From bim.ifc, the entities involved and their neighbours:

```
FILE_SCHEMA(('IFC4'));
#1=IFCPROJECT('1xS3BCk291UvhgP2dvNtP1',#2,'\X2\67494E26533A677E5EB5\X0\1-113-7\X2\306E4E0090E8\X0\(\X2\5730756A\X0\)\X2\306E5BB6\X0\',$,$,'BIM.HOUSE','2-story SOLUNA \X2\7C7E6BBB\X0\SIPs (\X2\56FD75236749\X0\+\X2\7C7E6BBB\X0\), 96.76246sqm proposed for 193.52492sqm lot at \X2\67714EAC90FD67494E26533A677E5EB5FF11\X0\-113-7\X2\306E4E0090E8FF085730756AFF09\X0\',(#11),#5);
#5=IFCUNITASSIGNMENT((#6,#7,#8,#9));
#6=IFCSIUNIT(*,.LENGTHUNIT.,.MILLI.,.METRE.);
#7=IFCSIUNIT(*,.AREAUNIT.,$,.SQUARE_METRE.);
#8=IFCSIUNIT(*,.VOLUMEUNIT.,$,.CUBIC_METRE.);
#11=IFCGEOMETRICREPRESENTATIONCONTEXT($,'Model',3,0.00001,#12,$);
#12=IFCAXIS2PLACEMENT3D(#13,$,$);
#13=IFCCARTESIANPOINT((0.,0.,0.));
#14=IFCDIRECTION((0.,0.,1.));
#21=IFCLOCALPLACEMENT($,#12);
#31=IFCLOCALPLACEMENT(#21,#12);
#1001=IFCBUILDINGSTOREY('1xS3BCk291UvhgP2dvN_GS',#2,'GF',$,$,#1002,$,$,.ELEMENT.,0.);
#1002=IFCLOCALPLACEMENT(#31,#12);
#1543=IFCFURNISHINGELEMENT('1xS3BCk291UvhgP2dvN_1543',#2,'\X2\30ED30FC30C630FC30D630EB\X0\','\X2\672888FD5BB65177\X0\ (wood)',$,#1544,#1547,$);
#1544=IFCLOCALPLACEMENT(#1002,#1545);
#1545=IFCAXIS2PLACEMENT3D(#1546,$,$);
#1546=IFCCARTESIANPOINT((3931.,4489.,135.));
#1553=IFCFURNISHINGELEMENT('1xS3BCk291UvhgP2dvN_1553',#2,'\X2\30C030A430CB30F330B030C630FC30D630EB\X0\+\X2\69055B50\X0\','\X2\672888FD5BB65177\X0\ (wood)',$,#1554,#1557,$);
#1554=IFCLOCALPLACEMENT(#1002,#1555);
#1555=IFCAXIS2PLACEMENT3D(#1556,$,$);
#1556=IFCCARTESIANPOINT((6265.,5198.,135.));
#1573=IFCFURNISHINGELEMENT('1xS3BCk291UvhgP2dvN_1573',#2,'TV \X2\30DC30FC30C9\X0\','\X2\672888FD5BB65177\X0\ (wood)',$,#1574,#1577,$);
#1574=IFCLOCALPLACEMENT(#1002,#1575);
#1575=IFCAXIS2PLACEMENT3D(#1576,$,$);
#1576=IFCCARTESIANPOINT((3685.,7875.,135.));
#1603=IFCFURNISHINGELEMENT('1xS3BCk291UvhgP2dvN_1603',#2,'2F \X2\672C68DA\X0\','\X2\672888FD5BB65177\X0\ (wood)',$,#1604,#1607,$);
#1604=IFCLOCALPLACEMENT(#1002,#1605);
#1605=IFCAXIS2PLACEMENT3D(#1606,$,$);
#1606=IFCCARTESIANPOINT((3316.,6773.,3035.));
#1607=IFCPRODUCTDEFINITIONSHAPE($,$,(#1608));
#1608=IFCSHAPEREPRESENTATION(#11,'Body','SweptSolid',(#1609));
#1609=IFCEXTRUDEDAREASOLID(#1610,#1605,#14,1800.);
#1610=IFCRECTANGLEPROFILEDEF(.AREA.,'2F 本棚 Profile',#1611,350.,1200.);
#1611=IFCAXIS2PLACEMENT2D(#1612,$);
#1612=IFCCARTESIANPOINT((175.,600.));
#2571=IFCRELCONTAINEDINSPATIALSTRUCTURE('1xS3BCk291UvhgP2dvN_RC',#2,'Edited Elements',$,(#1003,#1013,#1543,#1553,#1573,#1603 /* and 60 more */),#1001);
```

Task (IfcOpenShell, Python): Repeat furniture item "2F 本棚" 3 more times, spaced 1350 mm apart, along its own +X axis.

```python
import ifcopenshell
import ifcopenshell.api.geometry
import ifcopenshell.api.root
import ifcopenshell.util.element
import ifcopenshell.util.placement
import ifcopenshell.util.unit

model = ifcopenshell.open("bim.ifc")
unit_scale = ifcopenshell.util.unit.calculate_unit_scale(model)


def reuse_history(source, copy):
    """copy_class also copies each property set's owner history, people and application; keep the originals."""
    for rel in copy.IsDefinedBy:
        if rel.is_a("IfcRelDefinesByProperties") and (history := rel.RelatingPropertyDefinition.OwnerHistory):
            rel.RelatingPropertyDefinition.OwnerHistory = source.OwnerHistory
            ifcopenshell.util.element.remove_deep2(model, history)


source = model.by_guid("1xS3BCk291UvhgP2dvN_1603")
base = ifcopenshell.util.placement.get_local_placement(source.ObjectPlacement)
step = base[:3, 0] * 1.35 / unit_scale

for i in range(1, 4):
    copy = ifcopenshell.api.root.copy_class(model, product=source)
    copy.Representation = ifcopenshell.util.element.copy_deep(
        model, source.Representation, exclude=["IfcGeometricRepresentationContext", "IfcRepresentationMap"]
    )
    reuse_history(source, copy)
    matrix = base.copy()
    matrix[:3, 3] += i * step
    print("added at", matrix[:3, 3].round(3) + 0.0)
    ifcopenshell.api.geometry.edit_object_placement(model, product=copy, matrix=matrix, is_si=False)

model.write("bim_v2.ifc")
```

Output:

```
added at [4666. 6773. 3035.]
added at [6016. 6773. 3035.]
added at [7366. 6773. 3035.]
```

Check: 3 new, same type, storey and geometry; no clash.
